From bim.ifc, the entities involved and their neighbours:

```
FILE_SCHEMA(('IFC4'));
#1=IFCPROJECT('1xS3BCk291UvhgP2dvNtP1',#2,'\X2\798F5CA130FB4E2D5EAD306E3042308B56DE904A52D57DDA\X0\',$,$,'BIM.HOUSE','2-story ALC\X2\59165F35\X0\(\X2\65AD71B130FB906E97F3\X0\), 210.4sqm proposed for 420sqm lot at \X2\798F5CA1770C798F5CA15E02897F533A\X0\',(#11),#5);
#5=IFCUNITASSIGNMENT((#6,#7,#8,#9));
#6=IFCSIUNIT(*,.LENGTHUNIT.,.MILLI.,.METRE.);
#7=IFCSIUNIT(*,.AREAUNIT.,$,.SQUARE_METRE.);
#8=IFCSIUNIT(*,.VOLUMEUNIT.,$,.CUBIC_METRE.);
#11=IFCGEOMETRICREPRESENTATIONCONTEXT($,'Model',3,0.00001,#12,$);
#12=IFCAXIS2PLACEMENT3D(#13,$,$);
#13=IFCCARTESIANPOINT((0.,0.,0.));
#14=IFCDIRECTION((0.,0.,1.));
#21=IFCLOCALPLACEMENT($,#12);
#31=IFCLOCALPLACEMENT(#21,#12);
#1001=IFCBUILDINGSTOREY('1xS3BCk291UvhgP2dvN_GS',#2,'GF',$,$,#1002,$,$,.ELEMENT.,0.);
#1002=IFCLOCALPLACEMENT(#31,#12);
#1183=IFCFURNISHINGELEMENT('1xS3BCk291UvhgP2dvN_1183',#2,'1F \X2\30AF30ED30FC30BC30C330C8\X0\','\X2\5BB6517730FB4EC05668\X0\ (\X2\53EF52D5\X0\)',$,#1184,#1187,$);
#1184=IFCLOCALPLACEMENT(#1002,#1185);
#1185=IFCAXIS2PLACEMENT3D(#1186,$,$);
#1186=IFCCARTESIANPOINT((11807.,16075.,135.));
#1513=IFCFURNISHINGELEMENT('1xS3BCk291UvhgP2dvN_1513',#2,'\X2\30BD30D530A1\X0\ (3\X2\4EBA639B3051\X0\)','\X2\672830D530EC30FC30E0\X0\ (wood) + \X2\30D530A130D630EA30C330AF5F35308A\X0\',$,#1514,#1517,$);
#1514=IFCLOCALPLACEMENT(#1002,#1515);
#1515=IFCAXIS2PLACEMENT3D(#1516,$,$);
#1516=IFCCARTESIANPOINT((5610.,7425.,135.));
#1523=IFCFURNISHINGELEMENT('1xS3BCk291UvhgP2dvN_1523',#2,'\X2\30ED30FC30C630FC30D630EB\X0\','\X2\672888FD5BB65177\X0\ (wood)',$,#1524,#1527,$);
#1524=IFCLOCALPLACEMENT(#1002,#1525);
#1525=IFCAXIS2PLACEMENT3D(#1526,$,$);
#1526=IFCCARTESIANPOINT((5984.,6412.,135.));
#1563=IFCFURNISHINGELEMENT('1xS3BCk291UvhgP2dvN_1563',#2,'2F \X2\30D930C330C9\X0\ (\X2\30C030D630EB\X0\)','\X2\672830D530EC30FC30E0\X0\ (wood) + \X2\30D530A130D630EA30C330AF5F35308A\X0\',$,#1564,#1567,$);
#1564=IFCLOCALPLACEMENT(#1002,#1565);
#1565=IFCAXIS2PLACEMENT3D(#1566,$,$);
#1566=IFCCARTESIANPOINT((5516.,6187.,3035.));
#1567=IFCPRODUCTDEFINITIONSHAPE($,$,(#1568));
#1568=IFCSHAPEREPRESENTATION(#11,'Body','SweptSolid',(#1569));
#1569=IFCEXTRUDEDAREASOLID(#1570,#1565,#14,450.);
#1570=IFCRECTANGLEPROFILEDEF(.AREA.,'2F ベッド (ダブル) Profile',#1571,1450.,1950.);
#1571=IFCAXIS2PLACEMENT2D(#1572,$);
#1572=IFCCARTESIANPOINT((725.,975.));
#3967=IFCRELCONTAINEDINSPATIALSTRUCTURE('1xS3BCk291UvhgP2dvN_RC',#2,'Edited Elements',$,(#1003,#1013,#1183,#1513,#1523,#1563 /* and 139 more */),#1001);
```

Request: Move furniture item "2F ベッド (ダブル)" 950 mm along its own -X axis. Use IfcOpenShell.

```python
import ifcopenshell
import ifcopenshell.api.geometry
import ifcopenshell.util.placement
import ifcopenshell.util.unit

model = ifcopenshell.open("bim.ifc")
unit_scale = ifcopenshell.util.unit.calculate_unit_scale(model)

item = model.by_guid("1xS3BCk291UvhgP2dvN_1563")
matrix = ifcopenshell.util.placement.get_local_placement(item.ObjectPlacement)
matrix[:3, 3] -= matrix[:3, 0] * 0.95 / unit_scale
ifcopenshell.api.geometry.edit_object_placement(model, product=item, matrix=matrix, is_si=False)

print(ifcopenshell.util.placement.get_local_placement(item.ObjectPlacement).round(3) + 0.0)

model.write("bim_rev.ifc")
```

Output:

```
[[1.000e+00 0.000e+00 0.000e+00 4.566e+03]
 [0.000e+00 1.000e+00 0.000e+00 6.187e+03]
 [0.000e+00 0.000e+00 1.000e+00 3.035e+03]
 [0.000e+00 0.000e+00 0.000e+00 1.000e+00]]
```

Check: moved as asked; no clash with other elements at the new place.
